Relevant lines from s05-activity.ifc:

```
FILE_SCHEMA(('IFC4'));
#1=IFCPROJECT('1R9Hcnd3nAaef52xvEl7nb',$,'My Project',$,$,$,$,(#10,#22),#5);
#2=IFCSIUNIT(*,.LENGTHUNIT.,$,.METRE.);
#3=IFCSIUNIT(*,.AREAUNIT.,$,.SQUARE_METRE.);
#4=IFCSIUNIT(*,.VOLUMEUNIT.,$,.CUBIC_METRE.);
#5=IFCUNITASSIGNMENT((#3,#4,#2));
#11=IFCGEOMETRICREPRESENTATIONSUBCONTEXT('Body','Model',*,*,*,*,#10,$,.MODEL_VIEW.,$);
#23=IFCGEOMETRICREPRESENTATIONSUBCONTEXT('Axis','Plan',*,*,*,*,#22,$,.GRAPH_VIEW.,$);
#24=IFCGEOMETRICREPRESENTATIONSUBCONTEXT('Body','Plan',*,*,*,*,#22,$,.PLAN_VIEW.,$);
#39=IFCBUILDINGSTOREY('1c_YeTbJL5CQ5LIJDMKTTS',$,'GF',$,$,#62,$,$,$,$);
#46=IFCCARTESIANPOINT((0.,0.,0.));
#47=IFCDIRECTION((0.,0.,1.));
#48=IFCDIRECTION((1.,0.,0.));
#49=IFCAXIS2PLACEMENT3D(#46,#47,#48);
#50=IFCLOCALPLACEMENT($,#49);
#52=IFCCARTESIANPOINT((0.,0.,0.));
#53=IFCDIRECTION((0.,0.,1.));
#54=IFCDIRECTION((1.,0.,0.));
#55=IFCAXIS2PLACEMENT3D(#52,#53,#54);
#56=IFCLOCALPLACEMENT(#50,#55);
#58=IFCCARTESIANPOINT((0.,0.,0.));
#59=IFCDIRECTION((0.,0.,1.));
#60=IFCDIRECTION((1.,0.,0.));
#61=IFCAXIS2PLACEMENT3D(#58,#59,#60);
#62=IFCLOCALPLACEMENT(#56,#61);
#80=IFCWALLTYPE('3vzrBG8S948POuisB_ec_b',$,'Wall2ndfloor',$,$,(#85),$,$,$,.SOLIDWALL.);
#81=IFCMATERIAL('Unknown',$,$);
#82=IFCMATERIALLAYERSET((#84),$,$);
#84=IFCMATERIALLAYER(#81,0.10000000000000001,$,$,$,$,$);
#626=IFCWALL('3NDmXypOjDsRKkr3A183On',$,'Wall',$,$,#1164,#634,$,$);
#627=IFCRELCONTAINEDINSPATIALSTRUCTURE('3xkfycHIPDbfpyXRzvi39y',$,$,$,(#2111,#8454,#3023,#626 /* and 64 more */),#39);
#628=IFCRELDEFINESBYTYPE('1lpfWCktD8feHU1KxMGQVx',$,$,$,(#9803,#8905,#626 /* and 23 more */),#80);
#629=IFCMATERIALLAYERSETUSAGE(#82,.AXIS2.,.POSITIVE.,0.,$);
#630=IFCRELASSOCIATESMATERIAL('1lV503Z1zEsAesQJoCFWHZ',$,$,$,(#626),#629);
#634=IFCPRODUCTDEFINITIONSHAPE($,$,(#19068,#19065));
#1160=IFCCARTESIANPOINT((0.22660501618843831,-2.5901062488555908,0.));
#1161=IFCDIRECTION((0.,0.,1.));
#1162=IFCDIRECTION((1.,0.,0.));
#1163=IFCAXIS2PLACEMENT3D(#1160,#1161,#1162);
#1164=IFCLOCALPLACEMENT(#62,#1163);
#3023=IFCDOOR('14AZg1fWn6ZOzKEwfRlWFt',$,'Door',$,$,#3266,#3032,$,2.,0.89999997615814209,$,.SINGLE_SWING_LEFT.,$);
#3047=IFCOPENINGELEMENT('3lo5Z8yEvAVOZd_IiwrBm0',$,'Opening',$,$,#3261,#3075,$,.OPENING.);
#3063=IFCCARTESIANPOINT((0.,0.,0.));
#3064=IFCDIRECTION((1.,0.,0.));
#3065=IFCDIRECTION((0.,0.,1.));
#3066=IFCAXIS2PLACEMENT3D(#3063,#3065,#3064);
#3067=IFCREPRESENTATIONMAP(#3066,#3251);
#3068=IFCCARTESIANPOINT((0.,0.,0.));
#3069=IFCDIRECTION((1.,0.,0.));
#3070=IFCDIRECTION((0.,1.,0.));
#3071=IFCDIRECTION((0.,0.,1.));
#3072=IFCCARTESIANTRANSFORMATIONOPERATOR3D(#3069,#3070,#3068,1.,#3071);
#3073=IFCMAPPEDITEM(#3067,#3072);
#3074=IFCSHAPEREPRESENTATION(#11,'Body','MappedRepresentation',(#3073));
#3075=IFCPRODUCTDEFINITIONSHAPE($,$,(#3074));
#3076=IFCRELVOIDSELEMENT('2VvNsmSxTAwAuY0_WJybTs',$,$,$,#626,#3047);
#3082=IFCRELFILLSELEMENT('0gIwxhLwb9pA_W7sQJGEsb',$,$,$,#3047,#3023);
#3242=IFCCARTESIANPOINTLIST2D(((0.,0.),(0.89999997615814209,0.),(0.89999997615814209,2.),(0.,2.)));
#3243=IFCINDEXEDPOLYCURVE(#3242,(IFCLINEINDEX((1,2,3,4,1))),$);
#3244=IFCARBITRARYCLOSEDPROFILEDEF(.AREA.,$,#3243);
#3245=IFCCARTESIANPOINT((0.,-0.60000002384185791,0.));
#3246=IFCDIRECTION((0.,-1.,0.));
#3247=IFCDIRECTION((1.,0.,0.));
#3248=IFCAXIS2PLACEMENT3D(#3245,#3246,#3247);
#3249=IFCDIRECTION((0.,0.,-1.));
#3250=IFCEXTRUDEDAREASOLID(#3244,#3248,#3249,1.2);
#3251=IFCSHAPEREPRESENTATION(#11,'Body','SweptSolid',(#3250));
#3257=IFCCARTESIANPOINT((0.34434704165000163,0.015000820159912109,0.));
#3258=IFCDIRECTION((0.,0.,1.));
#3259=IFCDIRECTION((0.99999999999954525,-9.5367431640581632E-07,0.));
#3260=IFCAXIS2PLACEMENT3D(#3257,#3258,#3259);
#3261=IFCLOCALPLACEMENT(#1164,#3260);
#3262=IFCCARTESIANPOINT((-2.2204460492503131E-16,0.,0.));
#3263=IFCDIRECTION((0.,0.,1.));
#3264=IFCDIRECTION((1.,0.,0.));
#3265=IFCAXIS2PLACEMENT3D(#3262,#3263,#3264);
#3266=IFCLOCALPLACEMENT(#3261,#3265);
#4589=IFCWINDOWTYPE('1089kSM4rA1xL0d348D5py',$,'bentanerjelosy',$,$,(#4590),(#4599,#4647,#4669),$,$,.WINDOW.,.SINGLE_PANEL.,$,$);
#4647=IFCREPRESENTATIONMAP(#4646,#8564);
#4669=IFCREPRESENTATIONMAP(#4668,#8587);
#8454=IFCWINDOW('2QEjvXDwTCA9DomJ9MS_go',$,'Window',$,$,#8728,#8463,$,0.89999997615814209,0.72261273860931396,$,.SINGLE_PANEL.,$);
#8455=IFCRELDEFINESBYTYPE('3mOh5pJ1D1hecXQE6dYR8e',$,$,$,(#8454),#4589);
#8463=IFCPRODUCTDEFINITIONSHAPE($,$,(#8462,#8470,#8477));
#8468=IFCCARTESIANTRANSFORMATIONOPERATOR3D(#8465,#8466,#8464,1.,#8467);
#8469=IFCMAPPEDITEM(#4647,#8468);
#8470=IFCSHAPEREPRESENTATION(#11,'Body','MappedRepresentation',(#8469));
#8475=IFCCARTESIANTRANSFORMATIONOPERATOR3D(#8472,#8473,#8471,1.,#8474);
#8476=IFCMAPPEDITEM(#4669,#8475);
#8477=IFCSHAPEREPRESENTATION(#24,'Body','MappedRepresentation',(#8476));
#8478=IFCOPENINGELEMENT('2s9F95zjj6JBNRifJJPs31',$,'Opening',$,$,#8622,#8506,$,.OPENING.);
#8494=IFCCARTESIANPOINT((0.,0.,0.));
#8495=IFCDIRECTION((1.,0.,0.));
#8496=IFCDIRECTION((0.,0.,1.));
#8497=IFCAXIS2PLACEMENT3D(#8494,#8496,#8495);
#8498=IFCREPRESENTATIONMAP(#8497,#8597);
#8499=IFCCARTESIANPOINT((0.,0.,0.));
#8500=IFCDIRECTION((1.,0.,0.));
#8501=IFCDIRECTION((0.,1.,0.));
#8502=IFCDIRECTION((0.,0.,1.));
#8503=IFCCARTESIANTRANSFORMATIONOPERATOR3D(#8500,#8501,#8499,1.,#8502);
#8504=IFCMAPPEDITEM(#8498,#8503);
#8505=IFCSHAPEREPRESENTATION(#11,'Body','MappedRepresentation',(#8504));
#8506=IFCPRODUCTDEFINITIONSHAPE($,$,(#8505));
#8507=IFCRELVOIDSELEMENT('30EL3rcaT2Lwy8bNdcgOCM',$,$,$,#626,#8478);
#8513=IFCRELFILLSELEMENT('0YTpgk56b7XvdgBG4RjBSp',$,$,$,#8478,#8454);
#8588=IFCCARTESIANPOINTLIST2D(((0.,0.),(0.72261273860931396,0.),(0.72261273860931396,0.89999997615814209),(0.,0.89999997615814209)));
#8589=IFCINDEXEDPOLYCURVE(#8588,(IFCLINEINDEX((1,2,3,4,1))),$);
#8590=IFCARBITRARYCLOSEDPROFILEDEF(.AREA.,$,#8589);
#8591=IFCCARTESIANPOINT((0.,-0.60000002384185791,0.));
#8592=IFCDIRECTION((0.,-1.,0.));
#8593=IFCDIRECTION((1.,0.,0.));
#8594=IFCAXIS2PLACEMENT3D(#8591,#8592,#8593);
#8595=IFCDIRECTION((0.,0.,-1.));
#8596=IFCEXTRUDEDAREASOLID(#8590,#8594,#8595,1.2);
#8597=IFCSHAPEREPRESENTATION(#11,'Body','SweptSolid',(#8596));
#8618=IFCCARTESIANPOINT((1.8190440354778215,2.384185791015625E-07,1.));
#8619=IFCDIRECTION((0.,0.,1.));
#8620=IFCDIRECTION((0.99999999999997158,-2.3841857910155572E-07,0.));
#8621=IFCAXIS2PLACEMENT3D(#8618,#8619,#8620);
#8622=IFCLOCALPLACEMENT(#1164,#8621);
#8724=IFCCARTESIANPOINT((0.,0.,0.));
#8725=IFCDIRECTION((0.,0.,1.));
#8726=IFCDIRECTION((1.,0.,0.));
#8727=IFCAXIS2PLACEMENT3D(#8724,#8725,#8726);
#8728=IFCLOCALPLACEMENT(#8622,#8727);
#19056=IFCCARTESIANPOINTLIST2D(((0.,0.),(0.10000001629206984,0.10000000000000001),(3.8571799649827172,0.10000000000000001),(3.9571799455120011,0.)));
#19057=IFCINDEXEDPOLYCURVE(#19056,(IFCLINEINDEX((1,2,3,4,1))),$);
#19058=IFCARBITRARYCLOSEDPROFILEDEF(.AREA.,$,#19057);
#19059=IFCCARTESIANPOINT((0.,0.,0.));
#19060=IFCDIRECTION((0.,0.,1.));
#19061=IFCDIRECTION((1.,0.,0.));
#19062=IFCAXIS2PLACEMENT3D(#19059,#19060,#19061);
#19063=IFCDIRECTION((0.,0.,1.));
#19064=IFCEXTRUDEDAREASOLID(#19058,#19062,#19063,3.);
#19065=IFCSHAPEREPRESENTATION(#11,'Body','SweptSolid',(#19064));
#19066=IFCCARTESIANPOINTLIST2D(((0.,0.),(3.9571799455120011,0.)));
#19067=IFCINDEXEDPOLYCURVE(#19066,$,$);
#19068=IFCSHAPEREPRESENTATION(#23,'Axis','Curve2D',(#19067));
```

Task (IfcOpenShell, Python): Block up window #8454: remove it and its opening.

```python
import ifcopenshell
import ifcopenshell.api.feature
import ifcopenshell.api.root
import ifcopenshell.geom
import ifcopenshell.util.shape

model = ifcopenshell.open("s05-activity.ifc")
settings = ifcopenshell.geom.settings()


def volume(element):
    """Net volume in cubic metres, openings subtracted."""
    shape = ifcopenshell.geom.create_shape(settings, element)
    return ifcopenshell.util.shape.get_volume(shape.geometry)


window = model.by_guid("2QEjvXDwTCA9DomJ9MS_go")
opening = window.FillsVoids[0].RelatingOpeningElement
wall = opening.VoidsElements[0].RelatingBuildingElement
before = volume(wall)

ifcopenshell.api.root.remove_product(model, product=window)
ifcopenshell.api.feature.remove_feature(model, feature=opening)

after = volume(wall)

print(f"wall volume {before:.3f} -> {after:.3f} m3")

model.write("s05-activity-out.ifc")
```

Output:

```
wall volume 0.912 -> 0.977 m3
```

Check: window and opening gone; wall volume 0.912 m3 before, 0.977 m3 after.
